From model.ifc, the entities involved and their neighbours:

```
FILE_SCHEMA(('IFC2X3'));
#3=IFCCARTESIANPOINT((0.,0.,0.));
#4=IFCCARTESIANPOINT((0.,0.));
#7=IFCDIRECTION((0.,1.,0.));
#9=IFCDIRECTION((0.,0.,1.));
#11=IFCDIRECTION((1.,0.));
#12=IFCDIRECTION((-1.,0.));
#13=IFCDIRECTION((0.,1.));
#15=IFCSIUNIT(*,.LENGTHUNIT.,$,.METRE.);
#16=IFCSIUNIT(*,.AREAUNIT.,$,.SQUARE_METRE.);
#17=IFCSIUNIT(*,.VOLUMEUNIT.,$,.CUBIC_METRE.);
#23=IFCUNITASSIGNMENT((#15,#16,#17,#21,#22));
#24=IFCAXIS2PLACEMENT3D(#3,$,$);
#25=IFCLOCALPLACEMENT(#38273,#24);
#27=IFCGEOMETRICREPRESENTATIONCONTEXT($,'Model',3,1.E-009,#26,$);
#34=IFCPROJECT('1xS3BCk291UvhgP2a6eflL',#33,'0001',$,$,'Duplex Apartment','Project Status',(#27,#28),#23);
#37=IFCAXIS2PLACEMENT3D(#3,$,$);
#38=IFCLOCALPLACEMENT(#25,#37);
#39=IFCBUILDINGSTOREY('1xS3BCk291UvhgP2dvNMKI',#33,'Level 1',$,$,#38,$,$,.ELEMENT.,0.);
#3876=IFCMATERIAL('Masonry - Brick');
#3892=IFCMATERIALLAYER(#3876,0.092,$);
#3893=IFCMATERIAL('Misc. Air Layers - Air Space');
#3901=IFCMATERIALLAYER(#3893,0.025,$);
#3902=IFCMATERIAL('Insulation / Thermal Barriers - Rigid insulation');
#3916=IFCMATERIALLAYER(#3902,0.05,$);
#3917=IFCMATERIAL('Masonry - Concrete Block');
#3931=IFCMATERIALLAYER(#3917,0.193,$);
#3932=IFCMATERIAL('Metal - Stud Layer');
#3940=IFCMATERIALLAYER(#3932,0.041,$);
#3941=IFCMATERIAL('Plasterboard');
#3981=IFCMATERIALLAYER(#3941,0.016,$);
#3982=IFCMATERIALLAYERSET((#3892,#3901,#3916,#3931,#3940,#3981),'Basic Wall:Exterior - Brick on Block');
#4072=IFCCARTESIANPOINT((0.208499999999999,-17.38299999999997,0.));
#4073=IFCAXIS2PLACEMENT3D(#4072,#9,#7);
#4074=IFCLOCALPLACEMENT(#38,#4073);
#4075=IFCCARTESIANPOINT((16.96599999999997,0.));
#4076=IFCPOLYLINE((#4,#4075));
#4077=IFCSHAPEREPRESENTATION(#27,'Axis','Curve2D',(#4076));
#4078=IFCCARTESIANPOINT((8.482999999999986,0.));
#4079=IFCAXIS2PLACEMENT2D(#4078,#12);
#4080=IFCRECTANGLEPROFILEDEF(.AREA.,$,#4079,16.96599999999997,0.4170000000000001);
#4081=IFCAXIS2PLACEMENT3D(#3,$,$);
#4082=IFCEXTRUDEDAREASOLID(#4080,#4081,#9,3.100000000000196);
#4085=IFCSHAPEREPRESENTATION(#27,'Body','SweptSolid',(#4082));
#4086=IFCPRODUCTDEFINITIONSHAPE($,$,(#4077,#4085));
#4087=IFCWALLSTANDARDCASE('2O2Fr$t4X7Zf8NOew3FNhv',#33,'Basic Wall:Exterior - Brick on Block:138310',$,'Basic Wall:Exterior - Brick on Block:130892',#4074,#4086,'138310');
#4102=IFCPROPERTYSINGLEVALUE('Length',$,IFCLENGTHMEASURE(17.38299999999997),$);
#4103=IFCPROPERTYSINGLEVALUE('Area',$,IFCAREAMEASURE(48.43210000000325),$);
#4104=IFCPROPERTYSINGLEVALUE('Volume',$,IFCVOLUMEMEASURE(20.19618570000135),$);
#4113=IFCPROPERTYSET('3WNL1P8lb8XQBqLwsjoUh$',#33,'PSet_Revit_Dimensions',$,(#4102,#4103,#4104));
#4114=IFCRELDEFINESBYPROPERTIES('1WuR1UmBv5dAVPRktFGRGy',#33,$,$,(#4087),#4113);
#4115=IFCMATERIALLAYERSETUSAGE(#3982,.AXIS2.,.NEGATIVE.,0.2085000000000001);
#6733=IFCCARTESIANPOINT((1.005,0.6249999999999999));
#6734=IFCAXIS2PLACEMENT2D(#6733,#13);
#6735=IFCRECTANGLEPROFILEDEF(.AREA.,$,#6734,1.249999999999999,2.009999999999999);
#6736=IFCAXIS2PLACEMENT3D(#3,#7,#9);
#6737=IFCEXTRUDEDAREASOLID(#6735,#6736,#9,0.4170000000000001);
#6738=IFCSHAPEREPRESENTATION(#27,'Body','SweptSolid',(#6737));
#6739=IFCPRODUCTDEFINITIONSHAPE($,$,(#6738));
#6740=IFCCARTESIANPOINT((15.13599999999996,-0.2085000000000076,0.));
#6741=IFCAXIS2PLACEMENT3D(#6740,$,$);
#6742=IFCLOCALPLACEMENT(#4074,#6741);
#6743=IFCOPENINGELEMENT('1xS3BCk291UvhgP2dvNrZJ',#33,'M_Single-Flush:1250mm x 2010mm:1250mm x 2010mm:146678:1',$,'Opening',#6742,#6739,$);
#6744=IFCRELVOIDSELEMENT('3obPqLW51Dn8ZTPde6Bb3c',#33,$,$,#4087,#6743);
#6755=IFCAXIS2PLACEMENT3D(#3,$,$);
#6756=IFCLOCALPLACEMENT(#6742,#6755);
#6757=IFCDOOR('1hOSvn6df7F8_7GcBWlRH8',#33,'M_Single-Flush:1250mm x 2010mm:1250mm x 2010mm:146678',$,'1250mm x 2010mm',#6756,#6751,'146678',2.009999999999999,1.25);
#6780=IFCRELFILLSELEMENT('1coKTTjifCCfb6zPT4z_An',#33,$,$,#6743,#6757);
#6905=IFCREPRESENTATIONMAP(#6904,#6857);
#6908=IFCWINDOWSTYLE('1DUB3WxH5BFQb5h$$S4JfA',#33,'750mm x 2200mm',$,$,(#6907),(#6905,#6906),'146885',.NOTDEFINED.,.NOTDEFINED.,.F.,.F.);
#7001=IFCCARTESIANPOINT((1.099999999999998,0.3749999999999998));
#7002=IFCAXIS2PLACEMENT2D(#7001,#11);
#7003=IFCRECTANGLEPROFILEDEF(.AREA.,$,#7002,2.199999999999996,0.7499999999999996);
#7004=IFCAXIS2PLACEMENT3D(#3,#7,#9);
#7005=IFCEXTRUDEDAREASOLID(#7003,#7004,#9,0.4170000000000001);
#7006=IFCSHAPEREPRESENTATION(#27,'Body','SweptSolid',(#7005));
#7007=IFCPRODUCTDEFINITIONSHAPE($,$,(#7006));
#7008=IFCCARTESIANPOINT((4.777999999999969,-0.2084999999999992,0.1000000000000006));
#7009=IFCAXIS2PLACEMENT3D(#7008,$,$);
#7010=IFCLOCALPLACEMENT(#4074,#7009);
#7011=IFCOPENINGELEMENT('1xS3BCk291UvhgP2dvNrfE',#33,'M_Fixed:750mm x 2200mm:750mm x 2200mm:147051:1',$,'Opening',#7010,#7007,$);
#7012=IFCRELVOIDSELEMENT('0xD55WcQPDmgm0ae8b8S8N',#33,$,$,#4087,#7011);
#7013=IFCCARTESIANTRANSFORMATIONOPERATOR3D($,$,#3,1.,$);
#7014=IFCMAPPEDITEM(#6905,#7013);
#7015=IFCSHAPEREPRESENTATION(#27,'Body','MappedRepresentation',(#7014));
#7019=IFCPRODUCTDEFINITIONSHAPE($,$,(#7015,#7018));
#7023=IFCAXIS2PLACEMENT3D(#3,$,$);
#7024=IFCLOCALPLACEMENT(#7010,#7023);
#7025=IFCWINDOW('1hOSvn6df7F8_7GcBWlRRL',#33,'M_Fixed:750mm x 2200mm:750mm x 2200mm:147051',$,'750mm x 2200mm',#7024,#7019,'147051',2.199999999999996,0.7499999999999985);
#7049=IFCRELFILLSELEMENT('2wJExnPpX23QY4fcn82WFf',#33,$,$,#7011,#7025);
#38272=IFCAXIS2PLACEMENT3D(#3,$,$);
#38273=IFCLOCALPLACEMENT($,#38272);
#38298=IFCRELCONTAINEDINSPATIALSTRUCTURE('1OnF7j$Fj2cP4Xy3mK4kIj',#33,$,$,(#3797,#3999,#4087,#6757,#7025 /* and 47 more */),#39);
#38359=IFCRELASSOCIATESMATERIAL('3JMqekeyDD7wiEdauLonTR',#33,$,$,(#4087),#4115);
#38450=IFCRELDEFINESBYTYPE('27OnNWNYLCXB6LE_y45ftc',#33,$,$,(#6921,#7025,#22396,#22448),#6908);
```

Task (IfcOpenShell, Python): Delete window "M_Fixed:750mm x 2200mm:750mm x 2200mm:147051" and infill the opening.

```python
import ifcopenshell
import ifcopenshell.api.feature
import ifcopenshell.api.pset
import ifcopenshell.api.root
import ifcopenshell.geom
import ifcopenshell.util.element
import ifcopenshell.util.shape
import ifcopenshell.util.unit

model = ifcopenshell.open("model.ifc")
area_scale = ifcopenshell.util.unit.calculate_unit_scale(model, "AREAUNIT")
volume_scale = ifcopenshell.util.unit.calculate_unit_scale(model, "VOLUMEUNIT")
settings = ifcopenshell.geom.settings()


def volume(element):
    """Net volume in cubic metres, openings subtracted."""
    shape = ifcopenshell.geom.create_shape(settings, element)
    return ifcopenshell.util.shape.get_volume(shape.geometry)


window = model.by_guid("1hOSvn6df7F8_7GcBWlRRL")
opening = window.FillsVoids[0].RelatingOpeningElement
wall = opening.VoidsElements[0].RelatingBuildingElement
before = volume(wall)

ifcopenshell.api.root.remove_product(model, product=window)
ifcopenshell.api.feature.remove_feature(model, feature=opening)

after = volume(wall)
thickness = 0.417  # wall thickness in metres

# Update the wall's stored quantities.
pset = model.by_id(ifcopenshell.util.element.get_pset(wall, "PSet_Revit_Dimensions", should_inherit=False)["id"])
ifcopenshell.api.pset.edit_pset(model, pset=pset, properties={
    "Area": model.create_entity("IfcAreaMeasure", after / thickness / area_scale),
    "Volume": model.create_entity("IfcVolumeMeasure", after / volume_scale),
})

print(f"wall volume {before:.3f} -> {after:.3f} m3")

model.write("model_rev.ifc")
```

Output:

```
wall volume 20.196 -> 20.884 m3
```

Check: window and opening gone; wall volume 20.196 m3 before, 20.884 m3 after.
